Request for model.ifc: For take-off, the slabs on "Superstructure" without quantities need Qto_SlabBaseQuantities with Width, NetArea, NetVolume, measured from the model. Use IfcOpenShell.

First a look at what the model holds.

```python
import ifcopenshell
import ifcopenshell.util.element
import ifcopenshell.util.unit

model = ifcopenshell.open("model.ifc")
print(model.schema)
for unit_type in ("LENGTHUNIT", "AREAUNIT", "VOLUMEUNIT"):
    print(unit_type, ifcopenshell.util.unit.calculate_unit_scale(model, unit_type))
storey = next(s for s in model.by_type("IfcBuildingStorey") if s.Name == "Superstructure")
slabs = [e for e in ifcopenshell.util.element.get_decomposition(storey) if e.is_a("IfcSlab")]
for e in sorted(slabs, key=lambda e: e.id()):
    print(e.id(), e.is_a(), e.Name, list(ifcopenshell.util.element.get_psets(e, qtos_only=True)), sep=" | ")
```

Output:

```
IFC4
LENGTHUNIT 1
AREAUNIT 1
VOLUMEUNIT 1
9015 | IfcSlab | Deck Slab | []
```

```python
import ifcopenshell
import ifcopenshell.api.pset
import ifcopenshell.geom
import ifcopenshell.util.element
import ifcopenshell.util.shape
import ifcopenshell.util.unit

model = ifcopenshell.open("model.ifc")
unit_scale = ifcopenshell.util.unit.calculate_unit_scale(model)
area_scale = ifcopenshell.util.unit.calculate_unit_scale(model, "AREAUNIT")
volume_scale = ifcopenshell.util.unit.calculate_unit_scale(model, "VOLUMEUNIT")
settings = ifcopenshell.geom.settings()

storey = next(s for s in model.by_type("IfcBuildingStorey") if s.Name == "Superstructure")
slabs = [e for e in ifcopenshell.util.element.get_decomposition(storey) if e.is_a("IfcSlab")]

for e in sorted(slabs, key=lambda e: e.id()):
    if ifcopenshell.util.element.get_psets(e, qtos_only=True, should_inherit=False):
        continue
    # Geometry comes back in metres, in the element's own axes.
    shape = ifcopenshell.geom.create_shape(settings, e)
    values = {
        "Width": ifcopenshell.util.shape.get_z(shape.geometry) / unit_scale,
        "NetArea": ifcopenshell.util.shape.get_footprint_area(shape.geometry) / area_scale,
        "NetVolume": ifcopenshell.util.shape.get_volume(shape.geometry) / volume_scale,
    }
    qto = ifcopenshell.api.pset.add_qto(model, product=e, name="Qto_SlabBaseQuantities")
    ifcopenshell.api.pset.edit_qto(model, qto=qto, properties=values)
    print(e.id(), {k: round(v, 3) for k, v in values.items()})

model.write("model_edited.ifc")
```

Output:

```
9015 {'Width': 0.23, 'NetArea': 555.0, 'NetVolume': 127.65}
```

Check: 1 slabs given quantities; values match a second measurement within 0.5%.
